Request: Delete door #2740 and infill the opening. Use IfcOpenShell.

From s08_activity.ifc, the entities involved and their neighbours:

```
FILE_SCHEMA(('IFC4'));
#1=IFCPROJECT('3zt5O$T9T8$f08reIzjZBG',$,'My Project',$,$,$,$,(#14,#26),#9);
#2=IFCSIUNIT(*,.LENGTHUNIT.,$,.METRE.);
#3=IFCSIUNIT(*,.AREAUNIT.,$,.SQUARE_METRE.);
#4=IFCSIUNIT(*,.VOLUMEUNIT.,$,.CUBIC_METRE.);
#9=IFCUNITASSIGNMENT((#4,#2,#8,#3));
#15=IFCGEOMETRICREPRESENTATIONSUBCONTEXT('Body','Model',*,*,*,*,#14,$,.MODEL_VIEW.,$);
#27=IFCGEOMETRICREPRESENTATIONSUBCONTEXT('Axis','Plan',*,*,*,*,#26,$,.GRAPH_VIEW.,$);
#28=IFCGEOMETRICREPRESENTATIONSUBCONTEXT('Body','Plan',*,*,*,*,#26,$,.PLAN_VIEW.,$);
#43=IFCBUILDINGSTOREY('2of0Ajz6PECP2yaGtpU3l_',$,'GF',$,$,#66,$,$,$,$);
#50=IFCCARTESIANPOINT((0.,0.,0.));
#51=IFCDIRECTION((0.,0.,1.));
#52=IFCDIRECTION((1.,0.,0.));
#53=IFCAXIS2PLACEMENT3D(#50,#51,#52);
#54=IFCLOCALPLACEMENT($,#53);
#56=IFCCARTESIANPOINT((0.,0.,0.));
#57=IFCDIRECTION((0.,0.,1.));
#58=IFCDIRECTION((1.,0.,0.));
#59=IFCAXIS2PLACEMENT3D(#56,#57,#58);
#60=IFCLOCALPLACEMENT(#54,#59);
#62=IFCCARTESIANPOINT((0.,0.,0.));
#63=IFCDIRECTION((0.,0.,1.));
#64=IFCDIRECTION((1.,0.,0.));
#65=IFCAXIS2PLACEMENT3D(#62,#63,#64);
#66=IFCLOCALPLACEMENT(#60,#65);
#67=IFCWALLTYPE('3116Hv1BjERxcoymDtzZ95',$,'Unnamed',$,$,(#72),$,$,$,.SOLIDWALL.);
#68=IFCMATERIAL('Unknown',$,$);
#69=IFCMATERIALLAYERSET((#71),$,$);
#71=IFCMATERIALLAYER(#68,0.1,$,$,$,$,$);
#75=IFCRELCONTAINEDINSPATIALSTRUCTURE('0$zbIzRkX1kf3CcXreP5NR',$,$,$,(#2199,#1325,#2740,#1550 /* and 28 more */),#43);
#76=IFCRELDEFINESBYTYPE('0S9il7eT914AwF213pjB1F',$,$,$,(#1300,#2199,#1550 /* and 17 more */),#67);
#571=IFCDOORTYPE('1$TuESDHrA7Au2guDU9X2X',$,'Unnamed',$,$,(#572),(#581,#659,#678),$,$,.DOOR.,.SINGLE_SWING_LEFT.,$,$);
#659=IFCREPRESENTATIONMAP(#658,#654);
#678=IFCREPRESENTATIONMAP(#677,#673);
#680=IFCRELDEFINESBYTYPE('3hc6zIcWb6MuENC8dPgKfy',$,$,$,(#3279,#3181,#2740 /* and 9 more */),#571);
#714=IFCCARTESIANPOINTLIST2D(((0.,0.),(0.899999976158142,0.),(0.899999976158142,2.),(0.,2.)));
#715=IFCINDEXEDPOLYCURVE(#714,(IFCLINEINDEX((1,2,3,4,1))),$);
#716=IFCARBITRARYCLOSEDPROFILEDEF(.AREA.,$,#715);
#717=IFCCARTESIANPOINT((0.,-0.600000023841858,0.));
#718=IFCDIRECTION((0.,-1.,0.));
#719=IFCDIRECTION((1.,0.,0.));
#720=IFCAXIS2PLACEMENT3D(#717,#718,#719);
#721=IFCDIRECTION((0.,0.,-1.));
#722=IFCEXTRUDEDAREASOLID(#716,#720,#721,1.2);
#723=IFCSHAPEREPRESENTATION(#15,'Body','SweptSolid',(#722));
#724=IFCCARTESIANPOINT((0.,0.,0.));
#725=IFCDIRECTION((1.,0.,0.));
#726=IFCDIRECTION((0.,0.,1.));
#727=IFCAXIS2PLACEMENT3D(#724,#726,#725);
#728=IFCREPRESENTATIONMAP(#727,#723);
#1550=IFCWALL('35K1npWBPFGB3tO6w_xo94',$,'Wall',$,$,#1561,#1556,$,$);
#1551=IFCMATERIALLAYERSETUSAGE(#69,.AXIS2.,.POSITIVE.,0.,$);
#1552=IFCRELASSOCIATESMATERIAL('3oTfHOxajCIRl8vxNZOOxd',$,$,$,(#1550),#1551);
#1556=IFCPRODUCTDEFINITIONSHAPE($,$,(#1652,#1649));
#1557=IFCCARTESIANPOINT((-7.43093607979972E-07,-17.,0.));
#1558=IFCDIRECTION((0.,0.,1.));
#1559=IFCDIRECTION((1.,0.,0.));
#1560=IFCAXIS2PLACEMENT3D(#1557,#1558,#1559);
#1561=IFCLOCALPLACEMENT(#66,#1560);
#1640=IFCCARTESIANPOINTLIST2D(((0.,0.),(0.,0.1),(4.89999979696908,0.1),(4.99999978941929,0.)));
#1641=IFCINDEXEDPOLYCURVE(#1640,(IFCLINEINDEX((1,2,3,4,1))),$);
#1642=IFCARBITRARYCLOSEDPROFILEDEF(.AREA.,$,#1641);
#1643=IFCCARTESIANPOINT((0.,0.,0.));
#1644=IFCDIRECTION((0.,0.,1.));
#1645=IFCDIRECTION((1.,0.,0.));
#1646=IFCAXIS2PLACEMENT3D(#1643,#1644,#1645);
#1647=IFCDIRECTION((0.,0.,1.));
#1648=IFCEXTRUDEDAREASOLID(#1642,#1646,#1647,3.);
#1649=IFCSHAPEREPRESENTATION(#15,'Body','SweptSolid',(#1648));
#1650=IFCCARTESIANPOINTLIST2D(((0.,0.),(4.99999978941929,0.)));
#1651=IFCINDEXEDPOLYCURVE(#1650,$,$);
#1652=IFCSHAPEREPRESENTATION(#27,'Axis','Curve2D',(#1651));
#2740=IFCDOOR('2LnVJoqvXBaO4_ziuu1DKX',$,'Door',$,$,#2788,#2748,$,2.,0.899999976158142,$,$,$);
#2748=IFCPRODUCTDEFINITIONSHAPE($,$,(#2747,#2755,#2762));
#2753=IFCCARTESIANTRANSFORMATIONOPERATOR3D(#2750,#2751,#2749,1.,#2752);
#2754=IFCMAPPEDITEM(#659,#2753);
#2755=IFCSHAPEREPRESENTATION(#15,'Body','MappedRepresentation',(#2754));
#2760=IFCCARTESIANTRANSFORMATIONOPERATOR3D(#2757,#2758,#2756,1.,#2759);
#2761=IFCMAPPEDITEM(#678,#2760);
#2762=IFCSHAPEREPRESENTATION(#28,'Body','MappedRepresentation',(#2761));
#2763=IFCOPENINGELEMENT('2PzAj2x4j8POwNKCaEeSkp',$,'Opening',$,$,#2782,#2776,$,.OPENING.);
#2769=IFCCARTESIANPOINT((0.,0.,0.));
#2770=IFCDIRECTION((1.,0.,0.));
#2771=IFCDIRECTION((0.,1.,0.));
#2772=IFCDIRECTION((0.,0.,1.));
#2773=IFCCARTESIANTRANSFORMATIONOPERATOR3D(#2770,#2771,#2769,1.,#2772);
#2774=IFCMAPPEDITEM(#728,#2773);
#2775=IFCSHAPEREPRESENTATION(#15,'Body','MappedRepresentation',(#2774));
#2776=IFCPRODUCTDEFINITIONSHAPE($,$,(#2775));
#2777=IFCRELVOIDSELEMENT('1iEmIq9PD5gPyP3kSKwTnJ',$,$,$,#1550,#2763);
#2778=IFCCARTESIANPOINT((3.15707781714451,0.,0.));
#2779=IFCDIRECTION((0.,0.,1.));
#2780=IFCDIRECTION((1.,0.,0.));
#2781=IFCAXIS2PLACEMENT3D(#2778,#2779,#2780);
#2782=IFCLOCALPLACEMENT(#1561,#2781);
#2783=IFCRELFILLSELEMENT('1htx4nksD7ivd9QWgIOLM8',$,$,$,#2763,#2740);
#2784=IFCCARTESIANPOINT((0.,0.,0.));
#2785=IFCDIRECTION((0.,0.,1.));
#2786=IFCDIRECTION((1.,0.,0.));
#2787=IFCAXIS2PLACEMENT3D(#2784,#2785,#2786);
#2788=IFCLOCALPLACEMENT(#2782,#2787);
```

```python
import ifcopenshell
import ifcopenshell.api.feature
import ifcopenshell.api.root
import ifcopenshell.geom
import ifcopenshell.util.shape

model = ifcopenshell.open("s08_activity.ifc")
settings = ifcopenshell.geom.settings()


def volume(element):
    """Net volume in cubic metres, openings subtracted."""
    shape = ifcopenshell.geom.create_shape(settings, element)
    return ifcopenshell.util.shape.get_volume(shape.geometry)


door = model.by_guid("2LnVJoqvXBaO4_ziuu1DKX")
opening = door.FillsVoids[0].RelatingOpeningElement
wall = opening.VoidsElements[0].RelatingBuildingElement
before = volume(wall)

ifcopenshell.api.root.remove_product(model, product=door)
ifcopenshell.api.feature.remove_feature(model, feature=opening)

after = volume(wall)

print(f"wall volume {before:.3f} -> {after:.3f} m3")

model.write("s08_activity_rev.ifc")
```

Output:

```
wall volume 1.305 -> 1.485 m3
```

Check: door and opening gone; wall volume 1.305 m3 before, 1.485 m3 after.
